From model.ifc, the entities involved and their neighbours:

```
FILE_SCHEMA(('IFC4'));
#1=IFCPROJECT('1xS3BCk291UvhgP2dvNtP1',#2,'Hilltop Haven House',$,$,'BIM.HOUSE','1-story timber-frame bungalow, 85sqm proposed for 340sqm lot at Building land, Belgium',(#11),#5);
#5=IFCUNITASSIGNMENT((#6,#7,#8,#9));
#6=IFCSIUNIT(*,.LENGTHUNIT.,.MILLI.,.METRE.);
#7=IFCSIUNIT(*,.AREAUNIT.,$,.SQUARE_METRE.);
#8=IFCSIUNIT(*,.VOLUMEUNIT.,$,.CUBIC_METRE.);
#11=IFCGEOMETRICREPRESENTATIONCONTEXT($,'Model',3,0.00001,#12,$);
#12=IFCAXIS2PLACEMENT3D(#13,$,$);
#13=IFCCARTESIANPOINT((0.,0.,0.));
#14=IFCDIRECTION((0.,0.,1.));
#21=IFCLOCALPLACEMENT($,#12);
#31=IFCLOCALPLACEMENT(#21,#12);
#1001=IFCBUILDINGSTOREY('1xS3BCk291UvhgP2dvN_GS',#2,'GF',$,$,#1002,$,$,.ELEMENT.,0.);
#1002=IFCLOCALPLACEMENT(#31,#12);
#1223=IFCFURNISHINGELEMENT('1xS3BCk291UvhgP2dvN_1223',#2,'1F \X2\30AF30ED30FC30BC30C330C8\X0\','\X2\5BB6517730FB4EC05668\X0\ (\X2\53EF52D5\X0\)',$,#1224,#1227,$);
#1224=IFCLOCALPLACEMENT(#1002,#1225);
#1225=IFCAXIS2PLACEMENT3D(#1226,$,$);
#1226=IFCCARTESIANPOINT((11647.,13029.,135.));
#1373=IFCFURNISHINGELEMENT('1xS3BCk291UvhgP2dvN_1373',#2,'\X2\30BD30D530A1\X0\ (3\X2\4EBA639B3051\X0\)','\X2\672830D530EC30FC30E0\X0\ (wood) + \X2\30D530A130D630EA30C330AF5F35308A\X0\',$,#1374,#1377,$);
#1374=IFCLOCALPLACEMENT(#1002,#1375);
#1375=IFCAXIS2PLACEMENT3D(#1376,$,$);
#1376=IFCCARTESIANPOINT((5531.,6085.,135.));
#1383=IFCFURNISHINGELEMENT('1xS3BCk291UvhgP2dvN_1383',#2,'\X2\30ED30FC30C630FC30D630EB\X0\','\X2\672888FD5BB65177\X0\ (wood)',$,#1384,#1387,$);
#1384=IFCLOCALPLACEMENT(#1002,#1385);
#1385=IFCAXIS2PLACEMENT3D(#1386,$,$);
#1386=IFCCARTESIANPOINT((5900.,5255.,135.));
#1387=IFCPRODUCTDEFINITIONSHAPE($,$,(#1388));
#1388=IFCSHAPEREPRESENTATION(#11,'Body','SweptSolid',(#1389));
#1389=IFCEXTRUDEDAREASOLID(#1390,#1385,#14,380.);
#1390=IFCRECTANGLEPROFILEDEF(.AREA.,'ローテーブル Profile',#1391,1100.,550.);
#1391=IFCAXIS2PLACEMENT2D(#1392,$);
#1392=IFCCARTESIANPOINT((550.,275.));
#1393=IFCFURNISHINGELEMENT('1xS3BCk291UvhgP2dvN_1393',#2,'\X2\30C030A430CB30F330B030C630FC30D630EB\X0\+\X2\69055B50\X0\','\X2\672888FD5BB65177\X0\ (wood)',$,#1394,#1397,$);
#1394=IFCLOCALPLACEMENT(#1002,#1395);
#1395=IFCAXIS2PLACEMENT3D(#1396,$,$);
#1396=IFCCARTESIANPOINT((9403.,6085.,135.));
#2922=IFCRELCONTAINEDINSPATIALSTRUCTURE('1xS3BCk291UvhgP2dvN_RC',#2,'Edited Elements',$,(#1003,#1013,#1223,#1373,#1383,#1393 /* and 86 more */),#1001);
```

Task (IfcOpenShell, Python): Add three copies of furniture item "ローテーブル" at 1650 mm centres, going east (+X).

```python
import numpy as np
import ifcopenshell
import ifcopenshell.api.geometry
import ifcopenshell.api.root
import ifcopenshell.util.element
import ifcopenshell.util.placement
import ifcopenshell.util.unit

model = ifcopenshell.open("model.ifc")
unit_scale = ifcopenshell.util.unit.calculate_unit_scale(model)


def reuse_history(source, copy):
    """copy_class also copies each property set's owner history, people and application; keep the originals."""
    for rel in copy.IsDefinedBy:
        if rel.is_a("IfcRelDefinesByProperties") and (history := rel.RelatingPropertyDefinition.OwnerHistory):
            rel.RelatingPropertyDefinition.OwnerHistory = source.OwnerHistory
            ifcopenshell.util.element.remove_deep2(model, history)


source = model.by_id(1383)
base = ifcopenshell.util.placement.get_local_placement(source.ObjectPlacement)
step = np.array([1.0, 0.0, 0.0]) * 1.65 / unit_scale

for i in range(1, 4):
    copy = ifcopenshell.api.root.copy_class(model, product=source)
    copy.Representation = ifcopenshell.util.element.copy_deep(
        model, source.Representation, exclude=["IfcGeometricRepresentationContext", "IfcRepresentationMap"]
    )
    reuse_history(source, copy)
    matrix = base.copy()
    matrix[:3, 3] += i * step
    print("added at", matrix[:3, 3].round(3) + 0.0)
    ifcopenshell.api.geometry.edit_object_placement(model, product=copy, matrix=matrix, is_si=False)

model.write("model_edited.ifc")
```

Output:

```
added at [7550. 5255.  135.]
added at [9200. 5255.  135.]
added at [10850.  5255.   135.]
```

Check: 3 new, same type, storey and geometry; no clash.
